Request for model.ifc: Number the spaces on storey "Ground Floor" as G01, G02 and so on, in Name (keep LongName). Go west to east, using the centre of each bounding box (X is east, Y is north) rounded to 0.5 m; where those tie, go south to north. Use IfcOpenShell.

First a look at what the model holds.

```python
import ifcopenshell
import ifcopenshell.util.element
import ifcopenshell.util.placement

model = ifcopenshell.open("model.ifc")
print(model.schema)
storey = next(s for s in model.by_type("IfcBuildingStorey") if s.Name == "Ground Floor")
spaces = [e for e in ifcopenshell.util.element.get_decomposition(storey) if e.is_a("IfcSpace")]
for e in sorted(spaces, key=lambda e: e.id()):
    origin = ifcopenshell.util.placement.get_local_placement(e.ObjectPlacement)[:3, 3]
    print(e.id(), e.Name, e.LongName, origin.round(2) + 0.0, sep=" | ")
```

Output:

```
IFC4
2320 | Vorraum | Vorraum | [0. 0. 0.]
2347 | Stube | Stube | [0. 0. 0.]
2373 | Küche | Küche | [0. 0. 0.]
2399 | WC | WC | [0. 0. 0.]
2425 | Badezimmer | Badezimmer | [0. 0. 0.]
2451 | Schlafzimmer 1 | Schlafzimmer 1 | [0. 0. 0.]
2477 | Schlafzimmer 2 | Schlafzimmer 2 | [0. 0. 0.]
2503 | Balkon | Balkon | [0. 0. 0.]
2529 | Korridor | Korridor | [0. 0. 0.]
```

```python
import ifcopenshell
import ifcopenshell.geom
import ifcopenshell.util.element
import ifcopenshell.util.shape

model = ifcopenshell.open("model.ifc")
settings = ifcopenshell.geom.settings()
settings.set("use-world-coords", True)


def centre(element):
    shape = ifcopenshell.geom.create_shape(settings, element)
    return ifcopenshell.util.shape.get_bbox_centroid(shape.geometry)


storey = next(s for s in model.by_type("IfcBuildingStorey") if s.Name == "Ground Floor")
spaces = [e for e in ifcopenshell.util.element.get_decomposition(storey) if e.is_a("IfcSpace")]

# Insertion points can sit at a corner or the storey origin, so sort by the geometry (in metres).
centres = {e: centre(e) for e in spaces}
spaces.sort(key=lambda e: (round(centres[e][0] / 0.5), centres[e][1]))

for i, e in enumerate(spaces, start=1):
    number = f"G{i:02d}"
    e.Name = number
    print(e.id(), number)

model.write("model_updated.ifc")
```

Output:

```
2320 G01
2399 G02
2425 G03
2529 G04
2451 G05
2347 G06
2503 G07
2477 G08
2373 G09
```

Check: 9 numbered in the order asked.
